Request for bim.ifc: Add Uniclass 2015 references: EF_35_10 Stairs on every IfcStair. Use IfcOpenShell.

First a look at what the model holds.

```python
import ifcopenshell

model = ifcopenshell.open("bim.ifc")
print(model.schema)
print("classifications:", [c.Name for c in model.by_type("IfcClassification")])
for ifc_class in ("IfcDoor", "IfcRoof", "IfcStair", "IfcWall", "IfcWindow"):
    print(ifc_class, len(model.by_type(ifc_class)))
```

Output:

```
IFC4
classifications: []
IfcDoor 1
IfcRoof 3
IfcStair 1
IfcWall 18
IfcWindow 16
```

```python
import ifcopenshell
import ifcopenshell.api.classification

model = ifcopenshell.open("bim.ifc")

system = ifcopenshell.api.classification.add_classification(model, classification="Uniclass 2015")

codes = {
    "IfcStair": ("EF_35_10", "Stairs"),
}
for ifc_class, (code, name) in codes.items():
    products = model.by_type(ifc_class)
    ifcopenshell.api.classification.add_reference(
        model, products=products, classification=system, identification=code, name=name
    )
    print(code, len(products))

model.write("bim_rev.ifc")
```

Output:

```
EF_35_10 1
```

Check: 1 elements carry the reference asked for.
